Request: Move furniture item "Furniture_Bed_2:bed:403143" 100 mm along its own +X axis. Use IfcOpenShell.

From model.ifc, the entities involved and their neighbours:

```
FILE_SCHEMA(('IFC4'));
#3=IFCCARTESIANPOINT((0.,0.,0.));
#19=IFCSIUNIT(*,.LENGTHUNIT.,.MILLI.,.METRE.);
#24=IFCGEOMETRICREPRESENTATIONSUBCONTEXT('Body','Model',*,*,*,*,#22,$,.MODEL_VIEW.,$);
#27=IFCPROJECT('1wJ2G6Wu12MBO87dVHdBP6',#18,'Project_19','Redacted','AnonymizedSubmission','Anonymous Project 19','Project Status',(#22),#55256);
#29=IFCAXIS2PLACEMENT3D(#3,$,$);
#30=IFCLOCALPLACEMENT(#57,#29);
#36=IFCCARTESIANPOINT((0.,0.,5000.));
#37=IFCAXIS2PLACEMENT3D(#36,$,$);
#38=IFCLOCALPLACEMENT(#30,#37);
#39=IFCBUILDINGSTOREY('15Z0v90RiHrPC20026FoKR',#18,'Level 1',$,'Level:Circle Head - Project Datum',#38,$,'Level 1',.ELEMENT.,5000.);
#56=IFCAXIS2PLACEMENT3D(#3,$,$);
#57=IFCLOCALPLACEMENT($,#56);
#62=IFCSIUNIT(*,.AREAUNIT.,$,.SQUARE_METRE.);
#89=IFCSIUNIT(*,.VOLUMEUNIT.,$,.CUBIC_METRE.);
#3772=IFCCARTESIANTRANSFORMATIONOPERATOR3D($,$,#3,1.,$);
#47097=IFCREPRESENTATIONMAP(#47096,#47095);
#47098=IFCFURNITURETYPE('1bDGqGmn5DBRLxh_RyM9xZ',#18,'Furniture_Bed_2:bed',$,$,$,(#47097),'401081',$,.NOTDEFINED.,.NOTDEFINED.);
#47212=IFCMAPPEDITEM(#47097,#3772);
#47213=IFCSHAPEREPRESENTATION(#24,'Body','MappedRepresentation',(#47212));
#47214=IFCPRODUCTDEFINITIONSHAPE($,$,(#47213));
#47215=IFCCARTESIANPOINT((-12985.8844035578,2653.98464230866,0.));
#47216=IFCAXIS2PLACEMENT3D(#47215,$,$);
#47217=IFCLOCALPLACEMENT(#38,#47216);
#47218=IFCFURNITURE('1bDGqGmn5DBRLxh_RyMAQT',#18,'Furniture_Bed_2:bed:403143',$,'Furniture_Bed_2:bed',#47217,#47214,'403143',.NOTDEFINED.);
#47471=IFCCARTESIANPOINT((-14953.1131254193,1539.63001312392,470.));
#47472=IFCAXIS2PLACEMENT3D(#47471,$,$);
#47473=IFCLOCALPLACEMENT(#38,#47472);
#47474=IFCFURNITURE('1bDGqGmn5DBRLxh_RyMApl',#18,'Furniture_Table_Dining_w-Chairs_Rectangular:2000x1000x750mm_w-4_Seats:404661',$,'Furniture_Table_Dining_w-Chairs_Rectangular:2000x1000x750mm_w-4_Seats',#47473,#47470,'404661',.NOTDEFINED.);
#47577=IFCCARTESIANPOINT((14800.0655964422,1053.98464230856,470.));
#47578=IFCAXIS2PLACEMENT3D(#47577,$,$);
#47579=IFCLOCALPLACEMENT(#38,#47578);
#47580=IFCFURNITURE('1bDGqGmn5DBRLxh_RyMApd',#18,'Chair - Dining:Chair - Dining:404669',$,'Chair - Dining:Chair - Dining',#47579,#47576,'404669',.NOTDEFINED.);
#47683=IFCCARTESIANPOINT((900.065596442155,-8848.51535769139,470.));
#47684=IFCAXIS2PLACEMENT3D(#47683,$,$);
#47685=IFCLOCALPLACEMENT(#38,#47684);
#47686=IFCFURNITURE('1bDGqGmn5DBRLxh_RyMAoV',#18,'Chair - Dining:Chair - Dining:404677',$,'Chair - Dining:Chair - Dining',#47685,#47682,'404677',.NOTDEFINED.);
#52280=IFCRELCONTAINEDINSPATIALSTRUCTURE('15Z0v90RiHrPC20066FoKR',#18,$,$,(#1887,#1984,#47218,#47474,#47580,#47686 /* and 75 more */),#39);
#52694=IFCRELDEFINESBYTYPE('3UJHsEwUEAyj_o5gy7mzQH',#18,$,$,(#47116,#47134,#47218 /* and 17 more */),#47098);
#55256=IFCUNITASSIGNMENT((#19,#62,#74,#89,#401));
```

```python
import ifcopenshell
import ifcopenshell.api.geometry
import ifcopenshell.util.placement
import ifcopenshell.util.unit

model = ifcopenshell.open("model.ifc")
unit_scale = ifcopenshell.util.unit.calculate_unit_scale(model)

item = model.by_guid("1bDGqGmn5DBRLxh_RyMAQT")
matrix = ifcopenshell.util.placement.get_local_placement(item.ObjectPlacement)
matrix[:3, 3] += matrix[:3, 0] * 0.1 / unit_scale
ifcopenshell.api.geometry.edit_object_placement(model, product=item, matrix=matrix, is_si=False)

print(ifcopenshell.util.placement.get_local_placement(item.ObjectPlacement).round(3) + 0.0)

model.write("model_updated.ifc")
```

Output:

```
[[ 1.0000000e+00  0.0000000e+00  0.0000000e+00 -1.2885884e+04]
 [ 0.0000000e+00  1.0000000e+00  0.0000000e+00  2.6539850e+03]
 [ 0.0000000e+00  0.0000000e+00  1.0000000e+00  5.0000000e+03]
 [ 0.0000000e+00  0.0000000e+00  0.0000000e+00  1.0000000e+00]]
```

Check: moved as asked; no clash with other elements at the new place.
